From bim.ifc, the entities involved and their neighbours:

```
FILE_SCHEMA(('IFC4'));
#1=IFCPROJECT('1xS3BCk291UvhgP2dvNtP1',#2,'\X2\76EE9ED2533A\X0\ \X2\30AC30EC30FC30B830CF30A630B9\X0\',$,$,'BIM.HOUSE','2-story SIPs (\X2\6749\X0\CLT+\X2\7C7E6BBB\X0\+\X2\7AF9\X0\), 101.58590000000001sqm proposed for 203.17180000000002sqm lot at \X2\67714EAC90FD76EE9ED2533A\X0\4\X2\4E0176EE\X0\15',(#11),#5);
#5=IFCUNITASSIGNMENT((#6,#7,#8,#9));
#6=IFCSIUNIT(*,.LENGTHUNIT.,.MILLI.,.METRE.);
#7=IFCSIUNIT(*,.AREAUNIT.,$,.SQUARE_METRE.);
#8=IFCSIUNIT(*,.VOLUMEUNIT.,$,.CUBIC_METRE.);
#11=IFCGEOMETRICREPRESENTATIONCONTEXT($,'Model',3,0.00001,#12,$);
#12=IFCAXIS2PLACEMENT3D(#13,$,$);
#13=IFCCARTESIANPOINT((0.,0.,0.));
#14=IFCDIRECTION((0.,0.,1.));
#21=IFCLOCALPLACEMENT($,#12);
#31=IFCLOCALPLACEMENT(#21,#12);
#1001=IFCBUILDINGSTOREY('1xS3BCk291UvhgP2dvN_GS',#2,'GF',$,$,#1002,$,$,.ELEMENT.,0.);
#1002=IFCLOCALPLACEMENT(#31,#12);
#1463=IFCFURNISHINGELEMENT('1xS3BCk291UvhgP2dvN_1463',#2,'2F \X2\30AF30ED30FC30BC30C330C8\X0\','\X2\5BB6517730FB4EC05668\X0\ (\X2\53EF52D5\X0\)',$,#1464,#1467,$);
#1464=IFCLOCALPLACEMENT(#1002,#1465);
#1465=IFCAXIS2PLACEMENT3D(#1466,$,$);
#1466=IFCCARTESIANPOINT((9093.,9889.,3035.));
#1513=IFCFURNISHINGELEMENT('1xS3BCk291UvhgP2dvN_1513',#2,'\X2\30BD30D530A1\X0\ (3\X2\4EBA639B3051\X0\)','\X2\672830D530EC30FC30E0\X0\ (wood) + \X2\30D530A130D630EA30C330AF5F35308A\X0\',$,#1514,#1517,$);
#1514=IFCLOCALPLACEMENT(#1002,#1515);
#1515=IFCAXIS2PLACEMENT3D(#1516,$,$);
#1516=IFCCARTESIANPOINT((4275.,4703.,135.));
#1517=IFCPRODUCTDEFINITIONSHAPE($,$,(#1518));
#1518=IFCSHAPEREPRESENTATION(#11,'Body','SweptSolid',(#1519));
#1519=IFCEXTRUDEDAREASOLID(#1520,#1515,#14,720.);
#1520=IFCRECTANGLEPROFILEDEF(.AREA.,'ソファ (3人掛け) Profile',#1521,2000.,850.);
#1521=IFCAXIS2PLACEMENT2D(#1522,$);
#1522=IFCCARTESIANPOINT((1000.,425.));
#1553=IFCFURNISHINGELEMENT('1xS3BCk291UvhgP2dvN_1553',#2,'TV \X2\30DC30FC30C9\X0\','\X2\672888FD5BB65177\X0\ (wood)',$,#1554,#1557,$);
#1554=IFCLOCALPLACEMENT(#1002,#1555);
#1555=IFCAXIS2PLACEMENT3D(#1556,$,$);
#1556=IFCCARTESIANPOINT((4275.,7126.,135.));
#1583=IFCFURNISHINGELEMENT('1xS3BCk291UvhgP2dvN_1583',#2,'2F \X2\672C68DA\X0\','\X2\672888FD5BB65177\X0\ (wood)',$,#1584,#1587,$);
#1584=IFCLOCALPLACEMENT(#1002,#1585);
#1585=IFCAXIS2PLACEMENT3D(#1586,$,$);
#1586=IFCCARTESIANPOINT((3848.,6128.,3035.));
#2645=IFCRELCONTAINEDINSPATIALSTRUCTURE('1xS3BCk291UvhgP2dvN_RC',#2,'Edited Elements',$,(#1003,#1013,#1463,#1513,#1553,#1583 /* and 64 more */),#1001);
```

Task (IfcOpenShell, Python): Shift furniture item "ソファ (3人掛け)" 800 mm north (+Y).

```python
import ifcopenshell
import ifcopenshell.api.geometry
import ifcopenshell.util.placement

model = ifcopenshell.open("bim.ifc")

item = model.by_id(1513)
matrix = ifcopenshell.util.placement.get_local_placement(item.ObjectPlacement)
matrix[1, 3] += 800.0
ifcopenshell.api.geometry.edit_object_placement(model, product=item, matrix=matrix, is_si=False)

print(ifcopenshell.util.placement.get_local_placement(item.ObjectPlacement).round(3) + 0.0)

model.write("bim-out.ifc")
```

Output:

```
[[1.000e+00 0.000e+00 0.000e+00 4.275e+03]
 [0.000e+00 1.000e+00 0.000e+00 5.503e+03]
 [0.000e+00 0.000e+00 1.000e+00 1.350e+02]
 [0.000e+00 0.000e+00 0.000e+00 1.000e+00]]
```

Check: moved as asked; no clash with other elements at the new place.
